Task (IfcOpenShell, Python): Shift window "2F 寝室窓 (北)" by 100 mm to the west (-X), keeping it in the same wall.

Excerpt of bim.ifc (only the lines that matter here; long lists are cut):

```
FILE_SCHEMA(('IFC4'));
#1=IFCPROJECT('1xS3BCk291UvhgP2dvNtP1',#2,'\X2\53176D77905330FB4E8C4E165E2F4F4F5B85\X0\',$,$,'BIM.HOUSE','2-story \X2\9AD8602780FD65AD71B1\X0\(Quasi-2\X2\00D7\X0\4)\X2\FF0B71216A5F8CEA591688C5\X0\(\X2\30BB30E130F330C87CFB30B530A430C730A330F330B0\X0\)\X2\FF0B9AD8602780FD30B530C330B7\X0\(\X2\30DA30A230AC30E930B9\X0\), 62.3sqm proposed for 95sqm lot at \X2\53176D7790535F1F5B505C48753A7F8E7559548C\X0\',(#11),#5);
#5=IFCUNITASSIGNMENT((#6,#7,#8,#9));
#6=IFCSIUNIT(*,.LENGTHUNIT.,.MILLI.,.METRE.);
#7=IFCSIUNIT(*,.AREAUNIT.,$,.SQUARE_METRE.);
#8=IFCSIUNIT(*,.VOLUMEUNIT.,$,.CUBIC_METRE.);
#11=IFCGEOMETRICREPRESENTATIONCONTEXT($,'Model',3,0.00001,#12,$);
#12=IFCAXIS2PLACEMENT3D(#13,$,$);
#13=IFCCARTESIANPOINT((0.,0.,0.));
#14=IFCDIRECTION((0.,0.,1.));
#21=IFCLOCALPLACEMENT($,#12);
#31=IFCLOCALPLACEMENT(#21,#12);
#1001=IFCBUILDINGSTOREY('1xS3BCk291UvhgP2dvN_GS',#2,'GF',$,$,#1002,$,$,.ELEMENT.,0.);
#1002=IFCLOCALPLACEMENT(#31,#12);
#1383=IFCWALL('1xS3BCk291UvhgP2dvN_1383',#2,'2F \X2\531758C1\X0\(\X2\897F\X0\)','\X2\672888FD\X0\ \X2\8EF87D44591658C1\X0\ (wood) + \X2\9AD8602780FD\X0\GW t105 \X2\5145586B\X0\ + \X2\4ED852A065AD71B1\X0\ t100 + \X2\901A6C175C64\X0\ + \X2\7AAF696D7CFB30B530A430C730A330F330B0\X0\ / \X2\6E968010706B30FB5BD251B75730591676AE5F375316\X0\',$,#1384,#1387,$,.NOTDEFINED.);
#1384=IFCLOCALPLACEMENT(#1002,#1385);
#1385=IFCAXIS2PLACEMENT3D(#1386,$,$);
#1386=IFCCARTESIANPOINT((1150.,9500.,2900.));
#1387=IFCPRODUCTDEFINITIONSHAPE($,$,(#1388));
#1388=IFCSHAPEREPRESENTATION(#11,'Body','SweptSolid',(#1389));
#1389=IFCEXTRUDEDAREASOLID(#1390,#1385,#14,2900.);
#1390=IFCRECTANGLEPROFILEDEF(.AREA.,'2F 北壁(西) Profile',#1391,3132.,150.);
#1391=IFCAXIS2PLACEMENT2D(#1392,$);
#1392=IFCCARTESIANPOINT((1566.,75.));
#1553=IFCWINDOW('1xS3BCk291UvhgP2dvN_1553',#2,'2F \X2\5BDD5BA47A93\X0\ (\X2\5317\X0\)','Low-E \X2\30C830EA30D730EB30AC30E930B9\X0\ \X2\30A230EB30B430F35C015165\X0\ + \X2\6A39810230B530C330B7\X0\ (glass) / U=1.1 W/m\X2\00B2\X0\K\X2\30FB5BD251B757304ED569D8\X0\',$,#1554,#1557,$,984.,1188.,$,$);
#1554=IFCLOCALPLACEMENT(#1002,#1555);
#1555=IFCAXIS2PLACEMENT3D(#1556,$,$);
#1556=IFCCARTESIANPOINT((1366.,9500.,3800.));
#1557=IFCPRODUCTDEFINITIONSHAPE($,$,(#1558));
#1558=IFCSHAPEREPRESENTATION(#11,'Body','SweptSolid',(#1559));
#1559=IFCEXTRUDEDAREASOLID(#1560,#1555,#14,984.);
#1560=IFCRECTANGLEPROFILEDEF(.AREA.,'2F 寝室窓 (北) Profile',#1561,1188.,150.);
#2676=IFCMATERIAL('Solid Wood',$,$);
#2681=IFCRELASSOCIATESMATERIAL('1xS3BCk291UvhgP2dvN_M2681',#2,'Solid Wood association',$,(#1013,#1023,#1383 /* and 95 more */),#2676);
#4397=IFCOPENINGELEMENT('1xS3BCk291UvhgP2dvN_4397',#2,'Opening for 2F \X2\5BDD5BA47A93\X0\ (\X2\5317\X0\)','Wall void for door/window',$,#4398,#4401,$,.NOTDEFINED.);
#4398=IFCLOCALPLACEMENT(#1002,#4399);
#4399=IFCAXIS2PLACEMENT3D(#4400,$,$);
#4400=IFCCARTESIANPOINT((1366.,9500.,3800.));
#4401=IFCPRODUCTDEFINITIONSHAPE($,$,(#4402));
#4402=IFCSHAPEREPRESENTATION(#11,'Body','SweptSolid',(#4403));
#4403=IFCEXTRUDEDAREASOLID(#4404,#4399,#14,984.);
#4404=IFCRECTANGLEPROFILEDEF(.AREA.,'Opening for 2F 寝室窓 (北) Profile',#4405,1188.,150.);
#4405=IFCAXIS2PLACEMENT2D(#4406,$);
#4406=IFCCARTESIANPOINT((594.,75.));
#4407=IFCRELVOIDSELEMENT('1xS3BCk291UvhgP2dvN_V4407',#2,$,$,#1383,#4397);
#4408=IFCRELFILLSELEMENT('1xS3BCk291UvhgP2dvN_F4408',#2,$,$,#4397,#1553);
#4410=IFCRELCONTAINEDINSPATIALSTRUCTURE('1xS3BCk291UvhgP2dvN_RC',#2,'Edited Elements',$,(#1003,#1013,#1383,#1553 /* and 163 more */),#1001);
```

```python
import ifcopenshell
import ifcopenshell.api.geometry
import ifcopenshell.util.placement
import ifcopenshell.util.unit

model = ifcopenshell.open("bim.ifc")
unit_scale = ifcopenshell.util.unit.calculate_unit_scale(model)

window = model.by_guid("1xS3BCk291UvhgP2dvN_1553")
opening = window.FillsVoids[0].RelatingOpeningElement
wall = opening.VoidsElements[0].RelatingBuildingElement

wall_matrix = ifcopenshell.util.placement.get_local_placement(wall.ObjectPlacement)
shift = wall_matrix[:3, 0] * -0.1 / unit_scale
before = ifcopenshell.util.placement.get_local_placement(window.ObjectPlacement)[:3, 3].copy()

# The window is not placed relative to its opening, so move both.
for product in (opening, window):
    matrix = ifcopenshell.util.placement.get_local_placement(product.ObjectPlacement)
    matrix[:3, 3] += shift
    ifcopenshell.api.geometry.edit_object_placement(model, product=product, matrix=matrix, is_si=False)

after = ifcopenshell.util.placement.get_local_placement(window.ObjectPlacement)[:3, 3]
print("window moved by", (after - before).round(3) + 0.0)

model.write("bim_rev.ifc")
```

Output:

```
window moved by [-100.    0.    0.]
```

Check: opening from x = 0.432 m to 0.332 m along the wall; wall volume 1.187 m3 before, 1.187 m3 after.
